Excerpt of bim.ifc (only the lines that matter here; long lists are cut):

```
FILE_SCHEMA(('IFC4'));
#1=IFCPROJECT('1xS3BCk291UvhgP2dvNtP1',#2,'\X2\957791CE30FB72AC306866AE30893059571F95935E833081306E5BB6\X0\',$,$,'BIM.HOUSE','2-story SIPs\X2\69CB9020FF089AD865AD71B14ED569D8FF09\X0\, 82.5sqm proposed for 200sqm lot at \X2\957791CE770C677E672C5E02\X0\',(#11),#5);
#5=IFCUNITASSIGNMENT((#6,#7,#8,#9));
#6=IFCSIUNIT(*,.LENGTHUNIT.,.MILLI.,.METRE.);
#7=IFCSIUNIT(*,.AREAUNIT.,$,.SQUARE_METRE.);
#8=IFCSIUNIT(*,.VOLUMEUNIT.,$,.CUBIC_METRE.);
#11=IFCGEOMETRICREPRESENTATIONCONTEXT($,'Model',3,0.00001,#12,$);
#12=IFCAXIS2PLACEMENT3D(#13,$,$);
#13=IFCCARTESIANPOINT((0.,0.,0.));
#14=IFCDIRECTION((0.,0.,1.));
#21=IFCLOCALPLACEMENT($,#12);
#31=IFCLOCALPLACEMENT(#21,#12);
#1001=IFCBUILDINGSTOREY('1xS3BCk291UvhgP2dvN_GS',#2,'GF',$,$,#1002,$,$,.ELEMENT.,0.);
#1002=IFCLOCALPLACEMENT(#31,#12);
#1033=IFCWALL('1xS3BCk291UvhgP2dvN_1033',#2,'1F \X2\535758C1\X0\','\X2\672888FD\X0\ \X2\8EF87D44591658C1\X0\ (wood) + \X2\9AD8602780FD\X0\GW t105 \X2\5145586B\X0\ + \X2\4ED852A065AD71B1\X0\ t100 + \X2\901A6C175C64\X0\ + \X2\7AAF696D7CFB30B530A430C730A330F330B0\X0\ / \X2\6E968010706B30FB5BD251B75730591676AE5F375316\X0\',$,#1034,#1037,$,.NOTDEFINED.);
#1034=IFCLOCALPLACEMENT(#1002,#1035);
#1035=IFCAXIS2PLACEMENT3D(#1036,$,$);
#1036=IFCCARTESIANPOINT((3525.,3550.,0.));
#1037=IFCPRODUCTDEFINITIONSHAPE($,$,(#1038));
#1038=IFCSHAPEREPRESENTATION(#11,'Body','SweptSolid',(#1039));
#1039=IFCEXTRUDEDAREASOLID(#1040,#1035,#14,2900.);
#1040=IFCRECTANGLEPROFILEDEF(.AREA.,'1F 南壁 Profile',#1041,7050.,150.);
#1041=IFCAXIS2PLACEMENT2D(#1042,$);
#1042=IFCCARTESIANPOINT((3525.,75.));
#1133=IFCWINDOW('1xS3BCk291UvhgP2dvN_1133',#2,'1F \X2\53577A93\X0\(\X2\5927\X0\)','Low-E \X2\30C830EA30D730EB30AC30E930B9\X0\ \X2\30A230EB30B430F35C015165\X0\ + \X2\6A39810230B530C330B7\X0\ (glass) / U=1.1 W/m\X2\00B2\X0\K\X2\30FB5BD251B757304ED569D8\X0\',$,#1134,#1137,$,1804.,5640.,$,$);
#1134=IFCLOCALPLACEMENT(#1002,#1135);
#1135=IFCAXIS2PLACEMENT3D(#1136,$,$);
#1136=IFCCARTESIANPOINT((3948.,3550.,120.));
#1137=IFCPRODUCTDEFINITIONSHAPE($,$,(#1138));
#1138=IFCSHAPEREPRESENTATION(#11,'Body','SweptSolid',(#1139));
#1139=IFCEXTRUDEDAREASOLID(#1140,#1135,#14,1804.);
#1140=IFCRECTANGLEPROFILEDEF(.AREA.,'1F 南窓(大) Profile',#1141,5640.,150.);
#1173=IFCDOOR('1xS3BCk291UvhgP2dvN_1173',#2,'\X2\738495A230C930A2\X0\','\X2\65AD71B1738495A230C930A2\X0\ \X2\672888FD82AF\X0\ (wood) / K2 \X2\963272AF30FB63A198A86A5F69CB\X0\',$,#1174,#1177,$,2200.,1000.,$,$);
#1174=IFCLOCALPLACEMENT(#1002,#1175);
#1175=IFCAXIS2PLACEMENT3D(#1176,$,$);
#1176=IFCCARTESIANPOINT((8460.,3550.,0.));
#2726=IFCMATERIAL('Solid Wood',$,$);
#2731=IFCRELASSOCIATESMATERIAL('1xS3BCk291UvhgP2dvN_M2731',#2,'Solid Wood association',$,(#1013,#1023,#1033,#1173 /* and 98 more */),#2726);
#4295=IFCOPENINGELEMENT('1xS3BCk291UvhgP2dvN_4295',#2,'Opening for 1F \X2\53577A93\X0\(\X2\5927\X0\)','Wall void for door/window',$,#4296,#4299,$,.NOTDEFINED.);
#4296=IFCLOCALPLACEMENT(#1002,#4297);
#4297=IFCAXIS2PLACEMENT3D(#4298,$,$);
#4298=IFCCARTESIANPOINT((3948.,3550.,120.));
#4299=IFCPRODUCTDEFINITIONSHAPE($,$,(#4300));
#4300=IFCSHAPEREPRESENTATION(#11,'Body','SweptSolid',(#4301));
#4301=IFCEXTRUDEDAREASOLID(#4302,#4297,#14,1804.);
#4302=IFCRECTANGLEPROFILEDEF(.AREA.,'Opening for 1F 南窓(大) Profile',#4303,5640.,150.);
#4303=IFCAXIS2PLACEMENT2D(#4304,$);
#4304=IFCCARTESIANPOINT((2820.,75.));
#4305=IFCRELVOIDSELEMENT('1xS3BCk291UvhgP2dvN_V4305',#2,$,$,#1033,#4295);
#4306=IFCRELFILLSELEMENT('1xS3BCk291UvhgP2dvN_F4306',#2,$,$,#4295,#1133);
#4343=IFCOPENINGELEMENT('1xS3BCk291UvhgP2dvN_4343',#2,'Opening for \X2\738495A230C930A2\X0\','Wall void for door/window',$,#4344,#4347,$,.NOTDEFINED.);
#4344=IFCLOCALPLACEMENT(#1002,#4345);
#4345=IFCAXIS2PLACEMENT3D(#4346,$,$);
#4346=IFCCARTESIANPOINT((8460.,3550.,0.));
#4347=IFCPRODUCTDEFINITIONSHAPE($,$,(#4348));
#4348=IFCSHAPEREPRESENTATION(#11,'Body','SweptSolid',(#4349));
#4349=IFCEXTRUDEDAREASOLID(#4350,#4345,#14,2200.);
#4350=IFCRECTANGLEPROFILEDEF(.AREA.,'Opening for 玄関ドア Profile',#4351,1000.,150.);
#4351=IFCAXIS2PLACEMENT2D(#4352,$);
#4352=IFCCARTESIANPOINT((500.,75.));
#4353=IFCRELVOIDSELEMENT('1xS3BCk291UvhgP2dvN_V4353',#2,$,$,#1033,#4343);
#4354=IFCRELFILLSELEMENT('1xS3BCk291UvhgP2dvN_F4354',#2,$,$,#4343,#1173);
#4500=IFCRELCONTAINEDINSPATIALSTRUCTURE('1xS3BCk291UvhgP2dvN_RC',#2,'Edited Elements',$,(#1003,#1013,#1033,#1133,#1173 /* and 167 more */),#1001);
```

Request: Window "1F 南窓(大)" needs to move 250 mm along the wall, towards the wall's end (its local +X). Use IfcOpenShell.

```python
import ifcopenshell
import ifcopenshell.api.geometry
import ifcopenshell.util.placement
import ifcopenshell.util.unit

model = ifcopenshell.open("bim.ifc")
unit_scale = ifcopenshell.util.unit.calculate_unit_scale(model)

window = model.by_id(1133)
opening = window.FillsVoids[0].RelatingOpeningElement
wall = opening.VoidsElements[0].RelatingBuildingElement

wall_matrix = ifcopenshell.util.placement.get_local_placement(wall.ObjectPlacement)
shift = wall_matrix[:3, 0] * 0.25 / unit_scale
before = ifcopenshell.util.placement.get_local_placement(window.ObjectPlacement)[:3, 3].copy()

# The window is not placed relative to its opening, so move both.
for product in (opening, window):
    matrix = ifcopenshell.util.placement.get_local_placement(product.ObjectPlacement)
    matrix[:3, 3] += shift
    ifcopenshell.api.geometry.edit_object_placement(model, product=product, matrix=matrix, is_si=False)

after = ifcopenshell.util.placement.get_local_placement(window.ObjectPlacement)[:3, 3]
print("window moved by", (after - before).round(3) + 0.0)

model.write("bim-out.ifc")
```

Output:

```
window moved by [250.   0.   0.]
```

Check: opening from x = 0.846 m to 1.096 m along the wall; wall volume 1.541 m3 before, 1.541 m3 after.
